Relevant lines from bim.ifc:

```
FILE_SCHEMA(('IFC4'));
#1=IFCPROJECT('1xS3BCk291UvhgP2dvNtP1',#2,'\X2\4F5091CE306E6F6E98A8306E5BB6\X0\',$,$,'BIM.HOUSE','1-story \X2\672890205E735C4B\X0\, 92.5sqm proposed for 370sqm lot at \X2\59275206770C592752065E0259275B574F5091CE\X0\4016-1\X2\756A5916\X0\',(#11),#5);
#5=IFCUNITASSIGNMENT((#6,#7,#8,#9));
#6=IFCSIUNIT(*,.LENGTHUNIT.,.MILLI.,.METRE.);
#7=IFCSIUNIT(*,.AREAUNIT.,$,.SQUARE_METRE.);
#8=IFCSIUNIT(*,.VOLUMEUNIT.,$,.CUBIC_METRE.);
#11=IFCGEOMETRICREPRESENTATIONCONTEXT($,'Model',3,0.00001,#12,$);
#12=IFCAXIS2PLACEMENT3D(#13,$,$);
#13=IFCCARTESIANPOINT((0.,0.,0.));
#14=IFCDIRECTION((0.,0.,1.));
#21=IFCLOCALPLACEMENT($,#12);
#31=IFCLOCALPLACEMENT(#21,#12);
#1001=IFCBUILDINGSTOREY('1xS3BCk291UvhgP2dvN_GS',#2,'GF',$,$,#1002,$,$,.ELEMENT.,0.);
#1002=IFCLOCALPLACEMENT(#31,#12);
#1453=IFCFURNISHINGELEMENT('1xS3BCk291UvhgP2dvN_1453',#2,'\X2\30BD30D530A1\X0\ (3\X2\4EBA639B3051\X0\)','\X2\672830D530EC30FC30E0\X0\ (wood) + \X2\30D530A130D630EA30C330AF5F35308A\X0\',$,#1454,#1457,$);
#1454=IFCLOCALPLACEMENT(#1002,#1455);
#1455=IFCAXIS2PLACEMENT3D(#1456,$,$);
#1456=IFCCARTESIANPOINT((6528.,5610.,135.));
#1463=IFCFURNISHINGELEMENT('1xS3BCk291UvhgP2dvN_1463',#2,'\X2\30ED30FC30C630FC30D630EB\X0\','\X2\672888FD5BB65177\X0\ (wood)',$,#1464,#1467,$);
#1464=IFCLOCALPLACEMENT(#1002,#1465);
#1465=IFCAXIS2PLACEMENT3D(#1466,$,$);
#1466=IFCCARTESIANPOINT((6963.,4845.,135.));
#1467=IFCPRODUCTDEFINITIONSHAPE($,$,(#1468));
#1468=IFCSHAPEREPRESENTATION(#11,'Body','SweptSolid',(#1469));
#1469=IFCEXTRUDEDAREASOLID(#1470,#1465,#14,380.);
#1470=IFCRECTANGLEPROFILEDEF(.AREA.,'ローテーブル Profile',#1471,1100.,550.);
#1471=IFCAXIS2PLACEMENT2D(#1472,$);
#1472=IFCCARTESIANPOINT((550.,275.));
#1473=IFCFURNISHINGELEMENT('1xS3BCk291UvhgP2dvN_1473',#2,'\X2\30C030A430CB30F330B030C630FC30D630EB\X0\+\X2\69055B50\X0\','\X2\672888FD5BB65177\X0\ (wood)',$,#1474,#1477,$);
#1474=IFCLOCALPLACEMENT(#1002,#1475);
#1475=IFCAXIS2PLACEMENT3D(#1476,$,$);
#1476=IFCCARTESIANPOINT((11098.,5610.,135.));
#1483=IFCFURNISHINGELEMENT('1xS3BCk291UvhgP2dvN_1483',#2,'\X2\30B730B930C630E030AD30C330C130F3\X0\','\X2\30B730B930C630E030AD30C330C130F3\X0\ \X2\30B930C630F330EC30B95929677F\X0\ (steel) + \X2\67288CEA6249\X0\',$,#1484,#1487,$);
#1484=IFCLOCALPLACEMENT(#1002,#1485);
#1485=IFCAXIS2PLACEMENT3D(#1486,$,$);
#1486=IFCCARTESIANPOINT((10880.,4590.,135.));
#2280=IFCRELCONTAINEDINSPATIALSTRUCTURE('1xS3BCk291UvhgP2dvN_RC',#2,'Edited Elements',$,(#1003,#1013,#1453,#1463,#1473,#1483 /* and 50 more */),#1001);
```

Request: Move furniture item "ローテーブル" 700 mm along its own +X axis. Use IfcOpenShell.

```python
import ifcopenshell
import ifcopenshell.api.geometry
import ifcopenshell.util.placement

model = ifcopenshell.open("bim.ifc")

item = model.by_guid("1xS3BCk291UvhgP2dvN_1463")
matrix = ifcopenshell.util.placement.get_local_placement(item.ObjectPlacement)
matrix[:3, 3] += matrix[:3, 0] * 700.0
ifcopenshell.api.geometry.edit_object_placement(model, product=item, matrix=matrix, is_si=False)

print(ifcopenshell.util.placement.get_local_placement(item.ObjectPlacement).round(3) + 0.0)

model.write("bim_v2.ifc")
```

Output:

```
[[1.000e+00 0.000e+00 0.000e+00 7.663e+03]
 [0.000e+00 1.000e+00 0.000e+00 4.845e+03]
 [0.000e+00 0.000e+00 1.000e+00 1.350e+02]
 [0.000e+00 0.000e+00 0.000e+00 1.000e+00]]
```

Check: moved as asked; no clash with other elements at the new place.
